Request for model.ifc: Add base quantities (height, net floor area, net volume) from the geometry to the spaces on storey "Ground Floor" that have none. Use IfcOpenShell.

First a look at what the model holds.

```python
import ifcopenshell
import ifcopenshell.util.element
import ifcopenshell.util.unit

model = ifcopenshell.open("model.ifc")
print(model.schema)
for unit_type in ("LENGTHUNIT", "AREAUNIT", "VOLUMEUNIT"):
    print(unit_type, ifcopenshell.util.unit.calculate_unit_scale(model, unit_type))
storey = next(s for s in model.by_type("IfcBuildingStorey") if s.Name == "Ground Floor")
spaces = [e for e in ifcopenshell.util.element.get_decomposition(storey) if e.is_a("IfcSpace")]
for e in sorted(spaces, key=lambda e: e.id()):
    print(e.id(), e.is_a(), e.Name, list(ifcopenshell.util.element.get_psets(e, qtos_only=True)), sep=" | ")
```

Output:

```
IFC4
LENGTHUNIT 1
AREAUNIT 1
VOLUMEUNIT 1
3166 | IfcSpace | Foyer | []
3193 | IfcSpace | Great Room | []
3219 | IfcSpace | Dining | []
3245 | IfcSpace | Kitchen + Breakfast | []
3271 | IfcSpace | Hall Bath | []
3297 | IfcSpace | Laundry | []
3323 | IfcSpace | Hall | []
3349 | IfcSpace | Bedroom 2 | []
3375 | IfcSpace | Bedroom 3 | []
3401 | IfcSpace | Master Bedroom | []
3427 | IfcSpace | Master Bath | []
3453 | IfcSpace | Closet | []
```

```python
import ifcopenshell
import ifcopenshell.api.pset
import ifcopenshell.geom
import ifcopenshell.util.element
import ifcopenshell.util.shape
import ifcopenshell.util.unit

model = ifcopenshell.open("model.ifc")
unit_scale = ifcopenshell.util.unit.calculate_unit_scale(model)
area_scale = ifcopenshell.util.unit.calculate_unit_scale(model, "AREAUNIT")
volume_scale = ifcopenshell.util.unit.calculate_unit_scale(model, "VOLUMEUNIT")
settings = ifcopenshell.geom.settings()

storey = next(s for s in model.by_type("IfcBuildingStorey") if s.Name == "Ground Floor")
spaces = [e for e in ifcopenshell.util.element.get_decomposition(storey) if e.is_a("IfcSpace")]

for e in sorted(spaces, key=lambda e: e.id()):
    if ifcopenshell.util.element.get_psets(e, qtos_only=True, should_inherit=False):
        continue
    # Geometry comes back in metres, in the element's own axes.
    shape = ifcopenshell.geom.create_shape(settings, e)
    values = {
        "Height": ifcopenshell.util.shape.get_z(shape.geometry) / unit_scale,
        "NetFloorArea": ifcopenshell.util.shape.get_footprint_area(shape.geometry) / area_scale,
        "NetVolume": ifcopenshell.util.shape.get_volume(shape.geometry) / volume_scale,
    }
    qto = ifcopenshell.api.pset.add_qto(model, product=e, name="Qto_SpaceBaseQuantities")
    ifcopenshell.api.pset.edit_qto(model, qto=qto, properties=values)
    print(e.id(), {k: round(v, 3) for k, v in values.items()})

model.write("model_rev.ifc")
```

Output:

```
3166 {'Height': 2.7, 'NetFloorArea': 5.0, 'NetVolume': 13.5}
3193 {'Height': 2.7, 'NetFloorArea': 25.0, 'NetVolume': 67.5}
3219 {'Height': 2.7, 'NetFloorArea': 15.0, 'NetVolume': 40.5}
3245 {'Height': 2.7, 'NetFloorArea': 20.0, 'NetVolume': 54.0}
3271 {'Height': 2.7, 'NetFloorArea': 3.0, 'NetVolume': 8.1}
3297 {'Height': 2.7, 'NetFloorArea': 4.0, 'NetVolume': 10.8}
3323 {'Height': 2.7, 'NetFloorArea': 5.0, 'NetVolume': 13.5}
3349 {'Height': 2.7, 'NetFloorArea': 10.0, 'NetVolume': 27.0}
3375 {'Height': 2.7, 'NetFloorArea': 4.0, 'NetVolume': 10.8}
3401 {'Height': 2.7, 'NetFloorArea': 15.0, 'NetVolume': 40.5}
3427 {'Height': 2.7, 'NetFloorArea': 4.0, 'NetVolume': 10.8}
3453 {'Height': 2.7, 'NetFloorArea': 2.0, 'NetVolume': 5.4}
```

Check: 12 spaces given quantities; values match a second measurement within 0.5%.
